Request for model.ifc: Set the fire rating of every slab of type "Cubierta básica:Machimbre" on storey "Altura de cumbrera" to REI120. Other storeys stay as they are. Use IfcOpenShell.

First a look at what the model holds.

```python
import ifcopenshell
import ifcopenshell.util.element

model = ifcopenshell.open("model.ifc")
print(model.schema)
storey = next(s for s in model.by_type("IfcBuildingStorey") if s.Name == "Altura de cumbrera")
slabs = [e for e in ifcopenshell.util.element.get_decomposition(storey) if e.is_a("IfcSlab")]
seen = {}
for e in slabs:
    element_type = ifcopenshell.util.element.get_type(e)
    key = (element_type.Name if element_type != e and element_type else None, ifcopenshell.util.element.get_pset(e, "Pset_SlabCommon", "FireRating"))
    seen[key] = seen.get(key, 0) + 1
for (name, value), count in sorted(seen.items(), key=str):
    print(count, "x", name, "|", value)
```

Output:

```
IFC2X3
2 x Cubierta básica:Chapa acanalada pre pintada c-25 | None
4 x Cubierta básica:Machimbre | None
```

```python
import ifcopenshell
import ifcopenshell.api.pset
import ifcopenshell.util.element

model = ifcopenshell.open("model.ifc")

storey = next(s for s in model.by_type("IfcBuildingStorey") if s.Name == "Altura de cumbrera")
slabs = [e for e in ifcopenshell.util.element.get_decomposition(storey) if e.is_a("IfcSlab")]

count = 0
for e in slabs:
    element_type = ifcopenshell.util.element.get_type(e)
    if element_type in (None, e) or element_type.Name != "Cubierta básica:Machimbre":
        continue
    # add_pset returns the element's existing set when there is one.
    pset = ifcopenshell.api.pset.add_pset(model, product=e, name="Pset_SlabCommon")
    ifcopenshell.api.pset.edit_pset(model, pset=pset, properties={"FireRating": "REI120"})
    count += 1

print(count, "slabs updated")

model.write("model_updated.ifc")
```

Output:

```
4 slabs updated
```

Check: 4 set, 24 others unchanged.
